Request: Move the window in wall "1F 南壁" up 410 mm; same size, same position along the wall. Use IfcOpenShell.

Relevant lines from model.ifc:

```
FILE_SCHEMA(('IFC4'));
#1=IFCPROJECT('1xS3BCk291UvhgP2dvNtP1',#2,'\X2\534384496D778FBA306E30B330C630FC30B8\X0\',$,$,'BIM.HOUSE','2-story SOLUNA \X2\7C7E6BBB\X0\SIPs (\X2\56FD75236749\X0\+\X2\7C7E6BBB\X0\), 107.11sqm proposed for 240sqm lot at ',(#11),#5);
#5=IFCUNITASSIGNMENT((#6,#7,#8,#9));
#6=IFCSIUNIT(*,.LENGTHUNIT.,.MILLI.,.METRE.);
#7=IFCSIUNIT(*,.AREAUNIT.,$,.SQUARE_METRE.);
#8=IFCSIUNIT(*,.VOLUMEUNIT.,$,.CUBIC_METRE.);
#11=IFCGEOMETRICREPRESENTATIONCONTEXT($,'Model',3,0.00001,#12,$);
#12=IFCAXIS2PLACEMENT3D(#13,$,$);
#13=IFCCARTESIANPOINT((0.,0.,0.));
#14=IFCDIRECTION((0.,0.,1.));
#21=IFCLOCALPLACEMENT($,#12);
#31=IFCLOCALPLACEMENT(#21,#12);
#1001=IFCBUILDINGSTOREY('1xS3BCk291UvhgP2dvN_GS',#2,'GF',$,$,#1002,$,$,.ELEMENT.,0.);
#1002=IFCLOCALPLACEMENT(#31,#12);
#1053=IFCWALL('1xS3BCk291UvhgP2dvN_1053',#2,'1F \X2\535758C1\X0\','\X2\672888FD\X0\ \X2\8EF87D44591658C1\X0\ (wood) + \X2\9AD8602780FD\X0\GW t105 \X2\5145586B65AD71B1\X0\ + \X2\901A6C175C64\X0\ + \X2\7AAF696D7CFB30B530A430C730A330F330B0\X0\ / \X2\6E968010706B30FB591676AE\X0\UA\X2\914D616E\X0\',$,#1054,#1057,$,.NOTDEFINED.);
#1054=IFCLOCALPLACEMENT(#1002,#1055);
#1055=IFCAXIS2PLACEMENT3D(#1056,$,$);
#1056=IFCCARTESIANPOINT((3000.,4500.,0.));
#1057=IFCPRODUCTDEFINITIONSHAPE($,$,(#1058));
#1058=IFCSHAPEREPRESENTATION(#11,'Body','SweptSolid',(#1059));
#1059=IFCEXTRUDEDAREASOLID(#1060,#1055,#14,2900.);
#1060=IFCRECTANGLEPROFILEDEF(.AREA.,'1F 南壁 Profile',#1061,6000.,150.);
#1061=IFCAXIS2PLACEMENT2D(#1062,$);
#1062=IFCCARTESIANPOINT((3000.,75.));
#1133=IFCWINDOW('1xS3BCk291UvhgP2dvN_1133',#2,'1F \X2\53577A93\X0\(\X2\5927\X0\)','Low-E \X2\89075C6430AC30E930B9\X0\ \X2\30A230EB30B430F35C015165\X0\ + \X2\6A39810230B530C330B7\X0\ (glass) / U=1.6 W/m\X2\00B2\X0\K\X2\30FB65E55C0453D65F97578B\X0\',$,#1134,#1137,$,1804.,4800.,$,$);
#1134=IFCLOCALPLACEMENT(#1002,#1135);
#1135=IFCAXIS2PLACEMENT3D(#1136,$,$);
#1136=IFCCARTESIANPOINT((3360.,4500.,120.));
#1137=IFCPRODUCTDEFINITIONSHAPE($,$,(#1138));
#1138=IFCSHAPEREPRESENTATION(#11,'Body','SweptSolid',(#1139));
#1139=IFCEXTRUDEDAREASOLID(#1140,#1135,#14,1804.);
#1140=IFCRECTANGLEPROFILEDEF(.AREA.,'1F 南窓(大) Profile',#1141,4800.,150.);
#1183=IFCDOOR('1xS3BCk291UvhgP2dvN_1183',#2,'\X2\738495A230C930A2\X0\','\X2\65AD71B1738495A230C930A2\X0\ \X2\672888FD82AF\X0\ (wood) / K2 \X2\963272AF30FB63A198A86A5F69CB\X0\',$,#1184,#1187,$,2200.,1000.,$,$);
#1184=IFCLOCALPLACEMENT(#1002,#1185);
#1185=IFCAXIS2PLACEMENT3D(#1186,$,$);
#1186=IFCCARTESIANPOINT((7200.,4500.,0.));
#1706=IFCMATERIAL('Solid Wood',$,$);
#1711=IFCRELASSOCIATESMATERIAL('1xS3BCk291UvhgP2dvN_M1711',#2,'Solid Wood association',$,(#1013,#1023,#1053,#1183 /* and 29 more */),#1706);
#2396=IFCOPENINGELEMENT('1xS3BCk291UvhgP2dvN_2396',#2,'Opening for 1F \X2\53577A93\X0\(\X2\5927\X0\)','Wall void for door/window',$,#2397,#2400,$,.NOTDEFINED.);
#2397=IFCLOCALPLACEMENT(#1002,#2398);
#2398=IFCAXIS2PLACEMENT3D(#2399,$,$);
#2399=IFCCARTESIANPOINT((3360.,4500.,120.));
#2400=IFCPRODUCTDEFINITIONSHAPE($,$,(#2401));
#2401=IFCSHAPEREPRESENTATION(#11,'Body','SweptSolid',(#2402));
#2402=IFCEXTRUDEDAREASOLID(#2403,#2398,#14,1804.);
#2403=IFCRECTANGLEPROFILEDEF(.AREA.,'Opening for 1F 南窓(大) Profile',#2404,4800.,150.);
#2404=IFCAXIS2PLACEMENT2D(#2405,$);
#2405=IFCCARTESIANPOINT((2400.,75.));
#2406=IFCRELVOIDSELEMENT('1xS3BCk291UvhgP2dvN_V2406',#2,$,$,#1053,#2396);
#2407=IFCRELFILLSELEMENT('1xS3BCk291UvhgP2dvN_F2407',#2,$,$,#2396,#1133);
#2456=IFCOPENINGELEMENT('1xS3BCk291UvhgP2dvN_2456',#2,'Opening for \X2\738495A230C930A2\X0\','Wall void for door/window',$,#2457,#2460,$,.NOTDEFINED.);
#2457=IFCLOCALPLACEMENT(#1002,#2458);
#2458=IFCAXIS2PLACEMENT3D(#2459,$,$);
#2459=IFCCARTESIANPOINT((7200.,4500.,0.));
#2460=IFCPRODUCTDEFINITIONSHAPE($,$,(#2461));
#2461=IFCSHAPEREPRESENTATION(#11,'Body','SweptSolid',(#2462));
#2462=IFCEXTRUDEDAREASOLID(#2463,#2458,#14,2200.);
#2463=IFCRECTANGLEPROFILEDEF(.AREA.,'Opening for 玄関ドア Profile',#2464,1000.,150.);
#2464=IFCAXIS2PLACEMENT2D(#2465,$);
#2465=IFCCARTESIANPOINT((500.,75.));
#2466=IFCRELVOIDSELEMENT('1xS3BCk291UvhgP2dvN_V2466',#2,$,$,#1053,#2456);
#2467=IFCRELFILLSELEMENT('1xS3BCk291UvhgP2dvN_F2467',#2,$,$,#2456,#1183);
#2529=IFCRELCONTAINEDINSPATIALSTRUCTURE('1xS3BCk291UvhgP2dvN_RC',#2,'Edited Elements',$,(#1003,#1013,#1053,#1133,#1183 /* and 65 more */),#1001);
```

```python
import numpy as np
import ifcopenshell
import ifcopenshell.api.geometry
import ifcopenshell.util.placement
import ifcopenshell.util.unit

model = ifcopenshell.open("model.ifc")
unit_scale = ifcopenshell.util.unit.calculate_unit_scale(model)

window = model.by_guid("1xS3BCk291UvhgP2dvN_1133")
opening = window.FillsVoids[0].RelatingOpeningElement
dz = 0.41 / unit_scale

shift = np.array([0.0, 0.0, dz])
# The window is not placed relative to its opening, so move both.
for product in (opening, window):
    matrix = ifcopenshell.util.placement.get_local_placement(product.ObjectPlacement)
    matrix[:3, 3] += shift
    ifcopenshell.api.geometry.edit_object_placement(model, product=product, matrix=matrix, is_si=False)

print(f"moved by {dz * unit_scale:+.3f} m")

model.write("model_rev.ifc")
```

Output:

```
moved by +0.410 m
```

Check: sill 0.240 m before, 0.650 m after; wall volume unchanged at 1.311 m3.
